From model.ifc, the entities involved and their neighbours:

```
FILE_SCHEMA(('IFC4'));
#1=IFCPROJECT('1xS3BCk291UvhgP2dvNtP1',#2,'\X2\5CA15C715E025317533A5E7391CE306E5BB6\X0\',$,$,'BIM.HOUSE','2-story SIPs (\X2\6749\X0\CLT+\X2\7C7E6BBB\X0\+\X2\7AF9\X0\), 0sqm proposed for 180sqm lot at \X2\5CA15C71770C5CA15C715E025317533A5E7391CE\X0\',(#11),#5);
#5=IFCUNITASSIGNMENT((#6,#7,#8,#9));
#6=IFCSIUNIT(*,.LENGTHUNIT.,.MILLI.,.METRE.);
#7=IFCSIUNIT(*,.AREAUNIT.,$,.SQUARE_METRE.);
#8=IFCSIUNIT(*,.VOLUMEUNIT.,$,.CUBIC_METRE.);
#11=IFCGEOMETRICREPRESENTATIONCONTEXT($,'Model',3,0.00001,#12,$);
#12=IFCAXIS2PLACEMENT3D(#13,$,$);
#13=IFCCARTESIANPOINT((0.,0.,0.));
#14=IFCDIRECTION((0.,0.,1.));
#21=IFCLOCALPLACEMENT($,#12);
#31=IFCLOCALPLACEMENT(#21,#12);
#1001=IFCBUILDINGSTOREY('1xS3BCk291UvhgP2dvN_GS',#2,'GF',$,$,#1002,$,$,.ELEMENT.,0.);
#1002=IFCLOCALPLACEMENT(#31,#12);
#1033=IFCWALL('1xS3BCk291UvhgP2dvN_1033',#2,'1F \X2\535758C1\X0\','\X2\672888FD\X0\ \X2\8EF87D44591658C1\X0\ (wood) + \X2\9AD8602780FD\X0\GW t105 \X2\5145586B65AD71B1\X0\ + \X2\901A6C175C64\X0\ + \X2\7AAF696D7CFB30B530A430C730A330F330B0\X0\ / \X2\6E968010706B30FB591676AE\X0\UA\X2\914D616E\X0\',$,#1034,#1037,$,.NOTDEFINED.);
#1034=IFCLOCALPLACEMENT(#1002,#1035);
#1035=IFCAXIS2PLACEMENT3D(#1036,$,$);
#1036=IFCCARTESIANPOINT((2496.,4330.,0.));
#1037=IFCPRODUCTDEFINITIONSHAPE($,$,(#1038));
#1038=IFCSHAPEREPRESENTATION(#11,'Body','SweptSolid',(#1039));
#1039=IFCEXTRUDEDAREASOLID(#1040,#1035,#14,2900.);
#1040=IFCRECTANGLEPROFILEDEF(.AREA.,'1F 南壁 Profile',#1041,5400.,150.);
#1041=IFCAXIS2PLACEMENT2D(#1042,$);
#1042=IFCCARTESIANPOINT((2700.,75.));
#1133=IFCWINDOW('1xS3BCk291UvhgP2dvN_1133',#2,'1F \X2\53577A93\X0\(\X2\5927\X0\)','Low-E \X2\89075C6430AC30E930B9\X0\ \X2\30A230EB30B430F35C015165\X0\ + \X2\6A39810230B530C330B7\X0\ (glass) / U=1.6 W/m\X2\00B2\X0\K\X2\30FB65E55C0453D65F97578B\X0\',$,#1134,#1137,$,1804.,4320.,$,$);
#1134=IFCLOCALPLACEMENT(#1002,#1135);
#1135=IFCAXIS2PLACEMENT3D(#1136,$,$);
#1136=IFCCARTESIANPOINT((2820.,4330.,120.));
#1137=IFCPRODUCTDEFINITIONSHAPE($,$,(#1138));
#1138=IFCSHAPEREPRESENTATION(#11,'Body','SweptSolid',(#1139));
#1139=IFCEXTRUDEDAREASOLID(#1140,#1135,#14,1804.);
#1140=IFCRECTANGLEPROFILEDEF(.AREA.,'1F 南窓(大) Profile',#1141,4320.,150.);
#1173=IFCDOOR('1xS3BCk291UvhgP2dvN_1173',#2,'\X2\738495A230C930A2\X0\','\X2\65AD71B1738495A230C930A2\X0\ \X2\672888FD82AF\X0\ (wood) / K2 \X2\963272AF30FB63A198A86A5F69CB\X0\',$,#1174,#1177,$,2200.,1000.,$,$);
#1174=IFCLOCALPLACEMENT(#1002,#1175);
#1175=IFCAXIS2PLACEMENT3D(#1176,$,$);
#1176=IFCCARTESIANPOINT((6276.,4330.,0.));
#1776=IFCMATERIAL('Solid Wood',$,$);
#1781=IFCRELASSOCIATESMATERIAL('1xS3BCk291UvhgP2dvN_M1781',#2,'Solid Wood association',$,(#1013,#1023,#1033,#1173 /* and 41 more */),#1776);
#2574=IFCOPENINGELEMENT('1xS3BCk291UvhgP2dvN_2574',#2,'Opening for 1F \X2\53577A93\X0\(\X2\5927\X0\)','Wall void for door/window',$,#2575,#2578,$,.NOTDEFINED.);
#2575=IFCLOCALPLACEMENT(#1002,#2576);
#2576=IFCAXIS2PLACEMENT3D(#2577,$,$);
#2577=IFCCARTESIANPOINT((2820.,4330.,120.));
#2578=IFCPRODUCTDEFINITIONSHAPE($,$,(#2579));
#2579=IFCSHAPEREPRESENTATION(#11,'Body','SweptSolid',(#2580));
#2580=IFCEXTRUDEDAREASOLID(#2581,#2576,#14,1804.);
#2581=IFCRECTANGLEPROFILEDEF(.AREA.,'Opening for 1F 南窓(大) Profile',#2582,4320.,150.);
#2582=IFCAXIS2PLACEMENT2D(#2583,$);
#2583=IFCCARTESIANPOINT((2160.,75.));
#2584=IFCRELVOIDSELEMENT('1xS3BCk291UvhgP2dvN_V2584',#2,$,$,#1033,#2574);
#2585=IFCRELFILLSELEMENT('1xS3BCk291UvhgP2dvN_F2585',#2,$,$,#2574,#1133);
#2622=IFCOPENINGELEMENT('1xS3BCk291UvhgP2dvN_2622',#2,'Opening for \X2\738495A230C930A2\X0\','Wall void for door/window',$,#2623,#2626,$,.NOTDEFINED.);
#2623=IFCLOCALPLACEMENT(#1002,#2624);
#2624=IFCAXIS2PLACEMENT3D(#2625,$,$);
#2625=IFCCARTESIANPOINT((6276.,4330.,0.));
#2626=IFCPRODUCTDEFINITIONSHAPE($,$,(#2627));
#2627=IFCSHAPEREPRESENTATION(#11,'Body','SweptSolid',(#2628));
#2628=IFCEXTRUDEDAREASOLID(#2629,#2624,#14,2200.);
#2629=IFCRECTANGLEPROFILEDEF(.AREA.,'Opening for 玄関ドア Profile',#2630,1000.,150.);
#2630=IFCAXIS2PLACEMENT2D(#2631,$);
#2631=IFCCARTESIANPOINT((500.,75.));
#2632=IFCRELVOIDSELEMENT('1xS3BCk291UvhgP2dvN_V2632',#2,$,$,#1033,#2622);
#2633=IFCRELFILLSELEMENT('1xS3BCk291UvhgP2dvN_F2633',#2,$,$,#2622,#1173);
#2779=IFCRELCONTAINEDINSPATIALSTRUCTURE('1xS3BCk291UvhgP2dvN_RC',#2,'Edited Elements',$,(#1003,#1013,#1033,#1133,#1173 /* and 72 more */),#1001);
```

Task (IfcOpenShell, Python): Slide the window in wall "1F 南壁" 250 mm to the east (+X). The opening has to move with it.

```python
import ifcopenshell
import ifcopenshell.api.geometry
import ifcopenshell.util.placement
import ifcopenshell.util.unit

model = ifcopenshell.open("model.ifc")
unit_scale = ifcopenshell.util.unit.calculate_unit_scale(model)

window = model.by_guid("1xS3BCk291UvhgP2dvN_1133")
opening = window.FillsVoids[0].RelatingOpeningElement
wall = opening.VoidsElements[0].RelatingBuildingElement

wall_matrix = ifcopenshell.util.placement.get_local_placement(wall.ObjectPlacement)
shift = wall_matrix[:3, 0] * 0.25 / unit_scale
before = ifcopenshell.util.placement.get_local_placement(window.ObjectPlacement)[:3, 3].copy()

# The window is not placed relative to its opening, so move both.
for product in (opening, window):
    matrix = ifcopenshell.util.placement.get_local_placement(product.ObjectPlacement)
    matrix[:3, 3] += shift
    ifcopenshell.api.geometry.edit_object_placement(model, product=product, matrix=matrix, is_si=False)

after = ifcopenshell.util.placement.get_local_placement(window.ObjectPlacement)[:3, 3]
print("window moved by", (after - before).round(3) + 0.0)

model.write("model-out.ifc")
```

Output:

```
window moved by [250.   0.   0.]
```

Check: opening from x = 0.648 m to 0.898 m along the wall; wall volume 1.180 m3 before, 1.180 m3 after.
